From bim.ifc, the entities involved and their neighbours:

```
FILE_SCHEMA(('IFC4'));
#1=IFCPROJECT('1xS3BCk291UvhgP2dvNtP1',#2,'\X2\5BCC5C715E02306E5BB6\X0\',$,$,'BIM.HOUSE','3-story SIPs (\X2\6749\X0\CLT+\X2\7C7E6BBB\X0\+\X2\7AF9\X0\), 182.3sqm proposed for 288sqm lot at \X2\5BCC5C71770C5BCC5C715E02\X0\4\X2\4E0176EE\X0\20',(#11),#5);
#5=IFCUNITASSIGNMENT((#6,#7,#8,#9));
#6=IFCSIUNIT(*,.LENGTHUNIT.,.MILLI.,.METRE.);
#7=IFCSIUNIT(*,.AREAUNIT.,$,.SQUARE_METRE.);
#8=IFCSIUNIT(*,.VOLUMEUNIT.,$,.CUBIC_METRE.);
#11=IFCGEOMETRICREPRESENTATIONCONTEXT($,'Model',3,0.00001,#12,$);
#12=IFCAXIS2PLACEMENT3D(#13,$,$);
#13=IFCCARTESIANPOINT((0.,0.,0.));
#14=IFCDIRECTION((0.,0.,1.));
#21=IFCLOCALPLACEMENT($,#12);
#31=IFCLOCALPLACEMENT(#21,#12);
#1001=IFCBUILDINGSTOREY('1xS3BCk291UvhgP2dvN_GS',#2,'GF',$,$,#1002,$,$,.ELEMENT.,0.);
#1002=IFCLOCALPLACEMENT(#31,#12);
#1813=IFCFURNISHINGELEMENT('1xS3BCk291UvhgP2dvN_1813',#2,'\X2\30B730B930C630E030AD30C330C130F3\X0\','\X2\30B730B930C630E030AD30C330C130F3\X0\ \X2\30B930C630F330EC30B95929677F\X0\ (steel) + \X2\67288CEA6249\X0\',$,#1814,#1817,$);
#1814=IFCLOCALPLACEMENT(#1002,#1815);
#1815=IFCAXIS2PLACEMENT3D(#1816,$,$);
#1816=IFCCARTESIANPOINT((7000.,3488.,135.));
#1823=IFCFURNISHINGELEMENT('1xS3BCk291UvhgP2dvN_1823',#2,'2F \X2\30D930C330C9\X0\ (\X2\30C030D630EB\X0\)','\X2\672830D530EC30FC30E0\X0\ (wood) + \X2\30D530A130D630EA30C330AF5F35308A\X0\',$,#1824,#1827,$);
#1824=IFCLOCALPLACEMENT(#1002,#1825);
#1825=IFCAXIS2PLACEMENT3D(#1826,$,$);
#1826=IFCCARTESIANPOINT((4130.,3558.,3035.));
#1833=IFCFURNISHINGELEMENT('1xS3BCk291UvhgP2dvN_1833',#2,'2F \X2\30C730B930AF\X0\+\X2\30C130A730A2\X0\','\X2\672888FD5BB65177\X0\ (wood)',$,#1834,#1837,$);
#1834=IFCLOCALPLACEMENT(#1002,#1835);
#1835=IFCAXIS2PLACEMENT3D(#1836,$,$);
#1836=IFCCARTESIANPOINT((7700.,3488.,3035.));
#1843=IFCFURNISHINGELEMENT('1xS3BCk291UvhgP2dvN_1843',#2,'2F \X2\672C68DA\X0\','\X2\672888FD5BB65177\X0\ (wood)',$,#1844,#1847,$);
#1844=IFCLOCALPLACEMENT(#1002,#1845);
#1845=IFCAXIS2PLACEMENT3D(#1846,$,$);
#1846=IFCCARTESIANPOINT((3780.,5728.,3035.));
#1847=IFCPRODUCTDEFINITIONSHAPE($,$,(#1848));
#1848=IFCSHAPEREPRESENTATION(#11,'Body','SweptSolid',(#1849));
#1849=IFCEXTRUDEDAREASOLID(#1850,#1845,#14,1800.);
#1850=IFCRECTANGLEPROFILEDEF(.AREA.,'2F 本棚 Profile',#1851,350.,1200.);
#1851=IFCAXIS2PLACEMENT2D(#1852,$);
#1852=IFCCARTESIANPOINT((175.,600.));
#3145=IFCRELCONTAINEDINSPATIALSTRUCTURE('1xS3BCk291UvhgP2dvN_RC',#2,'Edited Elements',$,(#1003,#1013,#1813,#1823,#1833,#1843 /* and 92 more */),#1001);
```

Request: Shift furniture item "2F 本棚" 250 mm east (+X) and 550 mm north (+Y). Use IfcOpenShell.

```python
import ifcopenshell
import ifcopenshell.api.geometry
import ifcopenshell.util.placement

model = ifcopenshell.open("bim.ifc")

item = model.by_guid("1xS3BCk291UvhgP2dvN_1843")
matrix = ifcopenshell.util.placement.get_local_placement(item.ObjectPlacement)
matrix[0, 3] += 250.0
matrix[1, 3] += 550.0
ifcopenshell.api.geometry.edit_object_placement(model, product=item, matrix=matrix, is_si=False)

print(ifcopenshell.util.placement.get_local_placement(item.ObjectPlacement).round(3) + 0.0)

model.write("bim_v2.ifc")
```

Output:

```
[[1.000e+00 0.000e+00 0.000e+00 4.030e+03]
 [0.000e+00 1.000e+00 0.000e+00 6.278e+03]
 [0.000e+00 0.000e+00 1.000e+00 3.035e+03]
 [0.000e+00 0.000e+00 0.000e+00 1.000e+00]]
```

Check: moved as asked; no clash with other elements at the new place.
